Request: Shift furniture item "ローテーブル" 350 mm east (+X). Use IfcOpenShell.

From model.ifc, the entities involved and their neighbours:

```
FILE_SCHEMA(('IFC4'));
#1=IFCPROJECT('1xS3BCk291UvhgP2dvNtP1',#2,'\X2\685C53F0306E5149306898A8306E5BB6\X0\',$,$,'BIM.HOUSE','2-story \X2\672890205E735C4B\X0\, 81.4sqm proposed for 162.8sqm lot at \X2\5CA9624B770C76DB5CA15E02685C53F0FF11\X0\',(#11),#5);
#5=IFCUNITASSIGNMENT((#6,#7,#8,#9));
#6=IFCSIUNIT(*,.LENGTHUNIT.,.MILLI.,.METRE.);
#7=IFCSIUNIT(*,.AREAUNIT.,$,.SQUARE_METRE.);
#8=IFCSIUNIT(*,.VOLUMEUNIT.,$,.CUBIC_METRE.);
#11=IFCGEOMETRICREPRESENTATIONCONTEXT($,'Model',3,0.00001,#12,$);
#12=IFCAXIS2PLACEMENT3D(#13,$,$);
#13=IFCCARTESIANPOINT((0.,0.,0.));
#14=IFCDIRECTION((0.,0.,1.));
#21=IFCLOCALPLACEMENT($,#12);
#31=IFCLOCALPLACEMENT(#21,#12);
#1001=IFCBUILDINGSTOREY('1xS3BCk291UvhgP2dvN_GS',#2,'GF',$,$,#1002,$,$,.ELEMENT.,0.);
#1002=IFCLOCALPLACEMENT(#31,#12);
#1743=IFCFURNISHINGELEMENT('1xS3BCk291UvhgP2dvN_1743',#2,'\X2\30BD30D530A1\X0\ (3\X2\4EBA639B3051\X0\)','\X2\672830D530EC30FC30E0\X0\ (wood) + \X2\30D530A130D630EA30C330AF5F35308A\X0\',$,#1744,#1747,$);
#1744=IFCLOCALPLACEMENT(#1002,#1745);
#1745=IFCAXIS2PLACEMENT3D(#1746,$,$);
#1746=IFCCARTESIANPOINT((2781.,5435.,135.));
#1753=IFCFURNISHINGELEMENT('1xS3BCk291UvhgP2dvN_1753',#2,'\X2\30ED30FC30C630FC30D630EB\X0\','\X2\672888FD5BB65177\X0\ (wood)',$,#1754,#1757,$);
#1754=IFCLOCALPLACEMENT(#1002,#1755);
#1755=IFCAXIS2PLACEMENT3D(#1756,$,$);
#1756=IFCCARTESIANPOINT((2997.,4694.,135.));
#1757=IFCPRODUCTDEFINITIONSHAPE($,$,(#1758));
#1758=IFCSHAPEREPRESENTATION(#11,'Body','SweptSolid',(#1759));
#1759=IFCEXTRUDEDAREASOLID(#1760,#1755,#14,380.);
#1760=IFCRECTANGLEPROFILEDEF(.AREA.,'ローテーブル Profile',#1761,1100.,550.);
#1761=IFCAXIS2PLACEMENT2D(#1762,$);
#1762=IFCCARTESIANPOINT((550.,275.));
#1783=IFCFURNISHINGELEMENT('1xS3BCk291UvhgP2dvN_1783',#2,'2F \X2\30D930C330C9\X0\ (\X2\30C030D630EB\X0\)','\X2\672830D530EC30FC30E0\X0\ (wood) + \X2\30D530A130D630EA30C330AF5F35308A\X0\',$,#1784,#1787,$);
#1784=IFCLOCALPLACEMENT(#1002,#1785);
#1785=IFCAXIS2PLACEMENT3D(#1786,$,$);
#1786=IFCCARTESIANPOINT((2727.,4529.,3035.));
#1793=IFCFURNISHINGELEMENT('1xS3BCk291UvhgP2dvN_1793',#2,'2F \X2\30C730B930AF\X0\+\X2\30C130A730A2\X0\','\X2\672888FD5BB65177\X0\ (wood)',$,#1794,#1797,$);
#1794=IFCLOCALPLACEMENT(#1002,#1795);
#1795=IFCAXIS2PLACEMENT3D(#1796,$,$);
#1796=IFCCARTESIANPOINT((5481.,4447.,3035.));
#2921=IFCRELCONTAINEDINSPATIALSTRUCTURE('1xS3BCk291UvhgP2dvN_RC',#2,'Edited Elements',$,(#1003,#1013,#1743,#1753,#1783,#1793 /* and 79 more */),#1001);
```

```python
import ifcopenshell
import ifcopenshell.api.geometry
import ifcopenshell.util.placement
import ifcopenshell.util.unit

model = ifcopenshell.open("model.ifc")
unit_scale = ifcopenshell.util.unit.calculate_unit_scale(model)

item = model.by_guid("1xS3BCk291UvhgP2dvN_1753")
matrix = ifcopenshell.util.placement.get_local_placement(item.ObjectPlacement)
matrix[0, 3] += 0.35 / unit_scale
ifcopenshell.api.geometry.edit_object_placement(model, product=item, matrix=matrix, is_si=False)

print(ifcopenshell.util.placement.get_local_placement(item.ObjectPlacement).round(3) + 0.0)

model.write("model_updated.ifc")
```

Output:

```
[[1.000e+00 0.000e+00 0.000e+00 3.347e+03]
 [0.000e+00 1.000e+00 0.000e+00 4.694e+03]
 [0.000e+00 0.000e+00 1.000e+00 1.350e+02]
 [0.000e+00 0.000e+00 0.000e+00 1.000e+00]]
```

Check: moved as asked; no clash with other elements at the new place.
